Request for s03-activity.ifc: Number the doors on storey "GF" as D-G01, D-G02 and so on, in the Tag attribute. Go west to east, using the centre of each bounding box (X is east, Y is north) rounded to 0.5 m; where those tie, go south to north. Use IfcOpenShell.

First a look at what the model holds.

```python
import ifcopenshell
import ifcopenshell.util.element
import ifcopenshell.util.placement

model = ifcopenshell.open("s03-activity.ifc")
print(model.schema)
storey = next(s for s in model.by_type("IfcBuildingStorey") if s.Name == "GF")
doors = [e for e in ifcopenshell.util.element.get_decomposition(storey) if e.is_a("IfcDoor")]
for e in sorted(doors, key=lambda e: e.id()):
    origin = ifcopenshell.util.placement.get_local_placement(e.ObjectPlacement)[:3, 3]
    print(e.id(), e.Tag, e.Name, origin.round(2) + 0.0, sep=" | ")
```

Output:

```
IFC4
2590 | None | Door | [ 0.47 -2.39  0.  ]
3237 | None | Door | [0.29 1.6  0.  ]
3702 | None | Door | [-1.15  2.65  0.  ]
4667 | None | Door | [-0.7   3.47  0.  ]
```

```python
import ifcopenshell
import ifcopenshell.geom
import ifcopenshell.util.element
import ifcopenshell.util.shape

model = ifcopenshell.open("s03-activity.ifc")
settings = ifcopenshell.geom.settings()
settings.set("use-world-coords", True)


def centre(element):
    shape = ifcopenshell.geom.create_shape(settings, element)
    return ifcopenshell.util.shape.get_bbox_centroid(shape.geometry)


storey = next(s for s in model.by_type("IfcBuildingStorey") if s.Name == "GF")
doors = [e for e in ifcopenshell.util.element.get_decomposition(storey) if e.is_a("IfcDoor")]

# Insertion points can sit at a corner or the storey origin, so sort by the geometry (in metres).
centres = {e: centre(e) for e in doors}
doors.sort(key=lambda e: (round(centres[e][0] / 0.5), centres[e][1]))

for i, e in enumerate(doors, start=1):
    number = f"D-G{i:02d}"
    e.Tag = number
    print(e.id(), number)

model.write("s03-activity_rev.ifc")
```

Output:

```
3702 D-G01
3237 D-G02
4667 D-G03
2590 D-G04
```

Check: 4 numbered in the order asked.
